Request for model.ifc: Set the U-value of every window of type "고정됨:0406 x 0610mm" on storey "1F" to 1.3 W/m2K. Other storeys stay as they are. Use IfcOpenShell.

First a look at what the model holds.

```python
import ifcopenshell
import ifcopenshell.util.element

model = ifcopenshell.open("model.ifc")
print(model.schema)
storey = next(s for s in model.by_type("IfcBuildingStorey") if s.Name == "1F")
windows = [e for e in ifcopenshell.util.element.get_decomposition(storey) if e.is_a("IfcWindow")]
seen = {}
for e in windows:
    element_type = ifcopenshell.util.element.get_type(e)
    key = (element_type.Name if element_type != e and element_type else None, ifcopenshell.util.element.get_pset(e, "Pset_WindowCommon", "ThermalTransmittance"))
    seen[key] = seen.get(key, 0) + 1
for (name, value), count in sorted(seen.items(), key=str):
    print(count, "x", name, "|", value)
```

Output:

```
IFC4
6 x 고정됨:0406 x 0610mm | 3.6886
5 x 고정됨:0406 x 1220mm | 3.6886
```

```python
import ifcopenshell
import ifcopenshell.api.pset
import ifcopenshell.util.element

model = ifcopenshell.open("model.ifc")

storey = next(s for s in model.by_type("IfcBuildingStorey") if s.Name == "1F")
windows = [e for e in ifcopenshell.util.element.get_decomposition(storey) if e.is_a("IfcWindow")]

count = 0
for e in windows:
    element_type = ifcopenshell.util.element.get_type(e)
    if element_type in (None, e) or element_type.Name != "고정됨:0406 x 0610mm":
        continue
    # add_pset returns the element's existing set when there is one.
    pset = ifcopenshell.api.pset.add_pset(model, product=e, name="Pset_WindowCommon")
    ifcopenshell.api.pset.edit_pset(model, pset=pset, properties={"ThermalTransmittance": 1.3})
    count += 1

print(count, "windows updated")

model.write("model_edited.ifc")
```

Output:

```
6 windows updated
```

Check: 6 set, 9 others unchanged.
